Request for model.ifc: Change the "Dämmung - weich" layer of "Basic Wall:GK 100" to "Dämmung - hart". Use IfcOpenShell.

First a look at what the model holds.

```python
import ifcopenshell
import ifcopenshell.util.element

model = ifcopenshell.open("model.ifc")
print(model.schema)
for layer_set in model.by_type("IfcMaterialLayerSet"):
    if layer_set.LayerSetName == "Basic Wall:GK 100":
        for layer in layer_set.MaterialLayers:
            print(layer.id(), layer.Material and layer.Material.Name, layer.LayerThickness, sep=" | ")
        print(len(ifcopenshell.util.element.get_elements_by_material(model, layer_set)), "elements and types use it")
print(sorted(m.Name for m in model.by_type("IfcMaterial") if m.Name)[:60])
```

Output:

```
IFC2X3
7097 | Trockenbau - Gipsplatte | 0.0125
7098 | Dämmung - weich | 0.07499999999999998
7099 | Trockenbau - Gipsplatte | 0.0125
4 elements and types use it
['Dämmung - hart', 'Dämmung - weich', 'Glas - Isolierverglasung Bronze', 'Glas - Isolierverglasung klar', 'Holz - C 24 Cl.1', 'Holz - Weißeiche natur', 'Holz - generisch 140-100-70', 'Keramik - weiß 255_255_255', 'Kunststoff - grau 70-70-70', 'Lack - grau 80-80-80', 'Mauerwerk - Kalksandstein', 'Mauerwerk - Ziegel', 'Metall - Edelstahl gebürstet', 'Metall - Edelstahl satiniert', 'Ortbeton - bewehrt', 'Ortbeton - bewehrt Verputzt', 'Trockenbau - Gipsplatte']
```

```python
import ifcopenshell
import ifcopenshell.api.material

model = ifcopenshell.open("model.ifc")

layer_set = next(s for s in model.by_type("IfcMaterialLayerSet") if s.LayerSetName == "Basic Wall:GK 100")
layer = next(l for l in layer_set.MaterialLayers if l.Material and l.Material.Name == "Dämmung - weich")
material = next(m for m in model.by_type("IfcMaterial") if m.Name == "Dämmung - hart")

# Point this one layer at the other material; renaming the old one would change it everywhere.
ifcopenshell.api.material.edit_layer(model, layer=layer, attributes={}, material=material)

print([l.Material.Name if l.Material else None for l in layer_set.MaterialLayers])

model.write("model-out.ifc")
```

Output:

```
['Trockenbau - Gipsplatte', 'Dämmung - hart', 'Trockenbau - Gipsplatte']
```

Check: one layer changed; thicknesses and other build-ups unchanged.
